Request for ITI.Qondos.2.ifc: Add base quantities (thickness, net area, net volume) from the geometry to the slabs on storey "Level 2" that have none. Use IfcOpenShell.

First a look at what the model holds.

```python
import ifcopenshell
import ifcopenshell.util.element
import ifcopenshell.util.unit

model = ifcopenshell.open("ITI.Qondos.2.ifc")
print(model.schema)
for unit_type in ("LENGTHUNIT", "AREAUNIT", "VOLUMEUNIT"):
    print(unit_type, ifcopenshell.util.unit.calculate_unit_scale(model, unit_type))
storey = next(s for s in model.by_type("IfcBuildingStorey") if s.Name == "Level 2")
slabs = [e for e in ifcopenshell.util.element.get_decomposition(storey) if e.is_a("IfcSlab")]
for e in sorted(slabs, key=lambda e: e.id()):
    print(e.id(), e.is_a(), e.Name, list(ifcopenshell.util.element.get_psets(e, qtos_only=True)), sep=" | ")
```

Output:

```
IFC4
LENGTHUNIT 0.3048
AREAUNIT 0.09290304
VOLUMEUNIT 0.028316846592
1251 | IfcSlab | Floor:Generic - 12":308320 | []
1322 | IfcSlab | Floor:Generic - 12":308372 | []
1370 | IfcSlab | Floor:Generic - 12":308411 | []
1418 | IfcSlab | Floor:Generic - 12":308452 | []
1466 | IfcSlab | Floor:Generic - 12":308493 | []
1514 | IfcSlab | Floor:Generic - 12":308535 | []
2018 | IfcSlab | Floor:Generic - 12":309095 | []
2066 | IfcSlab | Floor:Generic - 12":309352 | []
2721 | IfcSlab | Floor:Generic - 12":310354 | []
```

```python
import ifcopenshell
import ifcopenshell.api.pset
import ifcopenshell.geom
import ifcopenshell.util.element
import ifcopenshell.util.shape
import ifcopenshell.util.unit

model = ifcopenshell.open("ITI.Qondos.2.ifc")
unit_scale = ifcopenshell.util.unit.calculate_unit_scale(model)
area_scale = ifcopenshell.util.unit.calculate_unit_scale(model, "AREAUNIT")
volume_scale = ifcopenshell.util.unit.calculate_unit_scale(model, "VOLUMEUNIT")
settings = ifcopenshell.geom.settings()

storey = next(s for s in model.by_type("IfcBuildingStorey") if s.Name == "Level 2")
slabs = [e for e in ifcopenshell.util.element.get_decomposition(storey) if e.is_a("IfcSlab")]

for e in sorted(slabs, key=lambda e: e.id()):
    if ifcopenshell.util.element.get_psets(e, qtos_only=True, should_inherit=False):
        continue
    # Geometry comes back in metres, in the element's own axes.
    shape = ifcopenshell.geom.create_shape(settings, e)
    values = {
        "Width": ifcopenshell.util.shape.get_z(shape.geometry) / unit_scale,
        "NetArea": ifcopenshell.util.shape.get_footprint_area(shape.geometry) / area_scale,
        "NetVolume": ifcopenshell.util.shape.get_volume(shape.geometry) / volume_scale,
    }
    qto = ifcopenshell.api.pset.add_qto(model, product=e, name="Qto_SlabBaseQuantities")
    ifcopenshell.api.pset.edit_qto(model, qto=qto, properties=values)
    print(e.id(), {k: round(v, 3) for k, v in values.items()})

model.write("ITI.Qondos.2_v2.ifc")
```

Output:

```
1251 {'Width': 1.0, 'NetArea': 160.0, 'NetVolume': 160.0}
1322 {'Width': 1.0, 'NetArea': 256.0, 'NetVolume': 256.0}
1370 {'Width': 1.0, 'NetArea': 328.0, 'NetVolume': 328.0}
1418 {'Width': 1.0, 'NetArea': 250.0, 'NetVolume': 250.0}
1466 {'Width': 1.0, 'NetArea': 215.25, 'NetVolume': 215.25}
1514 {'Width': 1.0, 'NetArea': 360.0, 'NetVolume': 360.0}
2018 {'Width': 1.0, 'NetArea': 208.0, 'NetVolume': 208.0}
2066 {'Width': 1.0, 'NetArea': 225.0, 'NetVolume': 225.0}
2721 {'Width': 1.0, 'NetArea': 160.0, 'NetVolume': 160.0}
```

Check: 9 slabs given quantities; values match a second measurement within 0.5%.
